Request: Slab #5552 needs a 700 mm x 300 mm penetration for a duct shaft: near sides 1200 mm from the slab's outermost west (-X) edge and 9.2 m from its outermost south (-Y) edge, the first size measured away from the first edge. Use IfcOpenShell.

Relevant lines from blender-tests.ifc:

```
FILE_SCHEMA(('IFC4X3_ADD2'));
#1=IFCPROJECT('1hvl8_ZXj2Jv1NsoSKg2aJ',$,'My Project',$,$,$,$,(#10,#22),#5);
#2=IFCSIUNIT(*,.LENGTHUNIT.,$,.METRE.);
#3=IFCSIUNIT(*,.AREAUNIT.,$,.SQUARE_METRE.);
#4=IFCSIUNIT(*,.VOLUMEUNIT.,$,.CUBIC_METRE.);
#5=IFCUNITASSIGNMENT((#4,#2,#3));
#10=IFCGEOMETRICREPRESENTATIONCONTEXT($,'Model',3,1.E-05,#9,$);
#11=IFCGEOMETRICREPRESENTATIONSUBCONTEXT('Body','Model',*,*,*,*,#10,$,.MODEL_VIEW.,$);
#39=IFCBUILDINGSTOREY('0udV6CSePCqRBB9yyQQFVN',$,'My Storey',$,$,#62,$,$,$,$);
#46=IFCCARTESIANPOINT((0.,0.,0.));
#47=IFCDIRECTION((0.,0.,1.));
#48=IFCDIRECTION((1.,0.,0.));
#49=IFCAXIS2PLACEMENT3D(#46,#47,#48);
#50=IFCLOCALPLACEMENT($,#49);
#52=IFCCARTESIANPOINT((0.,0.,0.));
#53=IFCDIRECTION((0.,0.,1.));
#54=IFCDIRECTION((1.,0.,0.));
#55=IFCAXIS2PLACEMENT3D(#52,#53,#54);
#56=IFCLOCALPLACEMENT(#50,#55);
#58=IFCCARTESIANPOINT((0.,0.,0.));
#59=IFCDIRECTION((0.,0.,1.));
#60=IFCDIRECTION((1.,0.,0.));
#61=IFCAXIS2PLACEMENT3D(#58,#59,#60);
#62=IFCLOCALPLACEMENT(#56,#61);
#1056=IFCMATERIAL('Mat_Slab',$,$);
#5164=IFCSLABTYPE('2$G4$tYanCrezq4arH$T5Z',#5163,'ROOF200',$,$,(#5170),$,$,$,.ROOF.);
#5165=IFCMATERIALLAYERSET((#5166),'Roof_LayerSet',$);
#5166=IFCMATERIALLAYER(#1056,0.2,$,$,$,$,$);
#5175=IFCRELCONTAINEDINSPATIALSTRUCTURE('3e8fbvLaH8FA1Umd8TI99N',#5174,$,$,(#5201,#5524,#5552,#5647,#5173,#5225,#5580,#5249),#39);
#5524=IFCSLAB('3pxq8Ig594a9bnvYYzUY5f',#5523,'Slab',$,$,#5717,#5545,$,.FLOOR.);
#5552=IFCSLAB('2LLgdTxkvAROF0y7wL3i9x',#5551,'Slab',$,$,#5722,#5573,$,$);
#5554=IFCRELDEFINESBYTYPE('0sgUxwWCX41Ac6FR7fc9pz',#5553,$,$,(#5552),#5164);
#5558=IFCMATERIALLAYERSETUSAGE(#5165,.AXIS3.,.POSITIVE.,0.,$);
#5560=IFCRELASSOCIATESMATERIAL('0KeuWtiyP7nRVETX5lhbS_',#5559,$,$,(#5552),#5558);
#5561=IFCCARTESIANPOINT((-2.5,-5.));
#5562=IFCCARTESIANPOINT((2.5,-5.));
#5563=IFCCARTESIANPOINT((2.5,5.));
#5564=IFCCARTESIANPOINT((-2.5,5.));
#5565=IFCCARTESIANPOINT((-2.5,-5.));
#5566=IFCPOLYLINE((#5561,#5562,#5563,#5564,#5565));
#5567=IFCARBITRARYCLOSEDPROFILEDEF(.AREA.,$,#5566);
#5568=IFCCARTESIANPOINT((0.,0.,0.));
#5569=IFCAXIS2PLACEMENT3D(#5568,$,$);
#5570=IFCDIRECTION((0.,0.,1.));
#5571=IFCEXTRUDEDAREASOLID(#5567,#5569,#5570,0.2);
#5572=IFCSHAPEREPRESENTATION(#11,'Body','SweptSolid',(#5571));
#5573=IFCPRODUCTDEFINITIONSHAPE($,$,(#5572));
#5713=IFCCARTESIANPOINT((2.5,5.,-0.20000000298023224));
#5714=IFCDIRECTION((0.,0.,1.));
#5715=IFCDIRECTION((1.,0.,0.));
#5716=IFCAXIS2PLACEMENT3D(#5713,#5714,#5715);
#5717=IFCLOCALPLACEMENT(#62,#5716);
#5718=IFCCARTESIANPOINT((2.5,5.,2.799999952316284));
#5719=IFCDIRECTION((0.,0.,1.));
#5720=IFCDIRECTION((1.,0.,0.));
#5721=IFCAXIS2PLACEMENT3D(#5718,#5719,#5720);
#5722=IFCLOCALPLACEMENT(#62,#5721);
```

```python
import numpy as np
import ifcopenshell
import ifcopenshell.api.feature
import ifcopenshell.api.geometry
import ifcopenshell.api.root
import ifcopenshell.geom
import ifcopenshell.util.placement
import ifcopenshell.util.representation
import ifcopenshell.util.shape
import ifcopenshell.util.unit

model = ifcopenshell.open("blender-tests.ifc")
unit_scale = ifcopenshell.util.unit.calculate_unit_scale(model)
settings = ifcopenshell.geom.settings()


def volume(element):
    """Net volume in cubic metres, openings subtracted."""
    shape = ifcopenshell.geom.create_shape(settings, element)
    return ifcopenshell.util.shape.get_volume(shape.geometry)


slab = model.by_guid("2LLgdTxkvAROF0y7wL3i9x")
before = volume(slab)

# Extent in the slab's own axes, in metres. The edges named are its -X and -Y sides.
slab_shape = ifcopenshell.geom.create_shape(settings, slab)
vertices = ifcopenshell.util.shape.get_vertices(slab_shape.geometry)
x_min, y_min, bottom = vertices.min(axis=0)
top = vertices[:, 2].max()

opening = ifcopenshell.api.root.create_entity(model, ifc_class="IfcOpeningElement", name="Duct shaft opening", predefined_type="OPENING")
context = ifcopenshell.util.representation.get_context(model, "Model", "Body", "MODEL_VIEW")
width, depth = 0.7, 0.3
outline = [(0.0, 0.0), (width, 0.0), (width, depth), (0.0, depth), (0.0, 0.0)]
# Overshoot both faces by 50 mm so the cut is clean.
shape = ifcopenshell.api.geometry.add_slab_representation(
    model, context=context, depth=top - bottom + 0.1, polyline=outline
)
ifcopenshell.api.geometry.assign_representation(model, product=opening, representation=shape)

matrix = ifcopenshell.util.placement.get_local_placement(slab.ObjectPlacement)
matrix[:, 3] = matrix @ np.append(np.array([x_min + 1.2, y_min + 9.2, bottom - 0.05]) / unit_scale, 1.0)
ifcopenshell.api.geometry.edit_object_placement(model, product=opening, matrix=matrix, is_si=False)
ifcopenshell.api.feature.add_feature(model, feature=opening, element=slab)

after = volume(slab)

print(f"slab volume {before:.3f} -> {after:.3f} m3")

model.write("blender-tests_edited.ifc")
```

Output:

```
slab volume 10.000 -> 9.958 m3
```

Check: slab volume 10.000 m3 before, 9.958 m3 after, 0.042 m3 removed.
